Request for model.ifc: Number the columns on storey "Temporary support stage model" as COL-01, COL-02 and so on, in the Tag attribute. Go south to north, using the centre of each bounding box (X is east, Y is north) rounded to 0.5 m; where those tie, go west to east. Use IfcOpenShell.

First a look at what the model holds.

```python
import ifcopenshell
import ifcopenshell.util.element
import ifcopenshell.util.placement

model = ifcopenshell.open("model.ifc")
print(model.schema)
storey = next(s for s in model.by_type("IfcBuildingStorey") if s.Name == "Temporary support stage model")
columns = [e for e in ifcopenshell.util.element.get_decomposition(storey) if e.is_a("IfcColumn")]
for e in sorted(columns, key=lambda e: e.id()):
    origin = ifcopenshell.util.placement.get_local_placement(e.ObjectPlacement)[:3, 3]
    print(e.id(), e.Tag, e.Name, origin.round(2) + 0.0, sep=" | ")
```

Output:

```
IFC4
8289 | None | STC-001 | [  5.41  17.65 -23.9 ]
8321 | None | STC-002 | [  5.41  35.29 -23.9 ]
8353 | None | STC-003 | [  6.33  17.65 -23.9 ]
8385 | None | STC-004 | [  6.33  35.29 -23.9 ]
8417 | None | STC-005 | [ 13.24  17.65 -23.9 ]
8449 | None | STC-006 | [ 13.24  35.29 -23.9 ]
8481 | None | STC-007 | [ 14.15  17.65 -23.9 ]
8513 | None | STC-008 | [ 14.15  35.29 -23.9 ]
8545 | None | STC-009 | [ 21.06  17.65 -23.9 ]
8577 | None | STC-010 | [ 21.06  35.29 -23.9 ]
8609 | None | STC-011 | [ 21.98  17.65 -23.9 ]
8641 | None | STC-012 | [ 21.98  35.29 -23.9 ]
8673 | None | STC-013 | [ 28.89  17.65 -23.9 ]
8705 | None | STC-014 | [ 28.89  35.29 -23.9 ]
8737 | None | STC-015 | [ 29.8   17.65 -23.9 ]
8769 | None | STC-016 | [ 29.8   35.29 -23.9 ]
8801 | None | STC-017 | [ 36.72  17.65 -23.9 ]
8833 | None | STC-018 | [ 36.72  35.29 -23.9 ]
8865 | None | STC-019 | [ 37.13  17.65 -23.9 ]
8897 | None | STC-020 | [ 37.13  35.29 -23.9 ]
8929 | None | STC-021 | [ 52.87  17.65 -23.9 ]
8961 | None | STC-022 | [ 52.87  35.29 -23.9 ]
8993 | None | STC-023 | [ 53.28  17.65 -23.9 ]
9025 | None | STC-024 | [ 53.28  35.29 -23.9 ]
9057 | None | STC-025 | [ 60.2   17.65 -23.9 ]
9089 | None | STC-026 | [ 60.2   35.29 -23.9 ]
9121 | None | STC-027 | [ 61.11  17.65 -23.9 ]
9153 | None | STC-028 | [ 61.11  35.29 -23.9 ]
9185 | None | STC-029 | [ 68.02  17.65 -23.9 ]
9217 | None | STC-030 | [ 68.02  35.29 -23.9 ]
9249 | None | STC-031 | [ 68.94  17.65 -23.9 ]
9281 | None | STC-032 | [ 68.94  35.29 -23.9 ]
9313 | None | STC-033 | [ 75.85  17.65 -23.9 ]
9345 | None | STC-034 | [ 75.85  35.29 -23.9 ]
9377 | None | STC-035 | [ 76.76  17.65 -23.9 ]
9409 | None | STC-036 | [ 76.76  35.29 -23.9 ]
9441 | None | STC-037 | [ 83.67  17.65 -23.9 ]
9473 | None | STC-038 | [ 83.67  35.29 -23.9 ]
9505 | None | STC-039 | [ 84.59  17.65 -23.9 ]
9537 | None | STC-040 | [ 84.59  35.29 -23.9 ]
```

```python
import ifcopenshell
import ifcopenshell.geom
import ifcopenshell.util.element
import ifcopenshell.util.shape

model = ifcopenshell.open("model.ifc")
settings = ifcopenshell.geom.settings()
settings.set("use-world-coords", True)


def centre(element):
    shape = ifcopenshell.geom.create_shape(settings, element)
    return ifcopenshell.util.shape.get_bbox_centroid(shape.geometry)


storey = next(s for s in model.by_type("IfcBuildingStorey") if s.Name == "Temporary support stage model")
columns = [e for e in ifcopenshell.util.element.get_decomposition(storey) if e.is_a("IfcColumn")]

# Insertion points can sit at a corner or the storey origin, so sort by the geometry (in metres).
centres = {e: centre(e) for e in columns}
columns.sort(key=lambda e: (round(centres[e][1] / 0.5), centres[e][0]))

for i, e in enumerate(columns, start=1):
    number = f"COL-{i:02d}"
    e.Tag = number
    print(e.id(), number)

model.write("model_updated.ifc")
```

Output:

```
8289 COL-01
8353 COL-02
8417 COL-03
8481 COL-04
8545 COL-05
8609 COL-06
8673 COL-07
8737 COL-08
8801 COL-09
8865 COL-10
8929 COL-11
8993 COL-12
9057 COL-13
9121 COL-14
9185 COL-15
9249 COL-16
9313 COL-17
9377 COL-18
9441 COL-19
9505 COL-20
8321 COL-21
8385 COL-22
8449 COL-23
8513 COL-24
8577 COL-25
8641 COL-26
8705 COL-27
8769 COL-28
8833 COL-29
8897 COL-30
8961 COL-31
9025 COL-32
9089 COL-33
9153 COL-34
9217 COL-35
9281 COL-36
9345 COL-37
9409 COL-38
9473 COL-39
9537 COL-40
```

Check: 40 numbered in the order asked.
